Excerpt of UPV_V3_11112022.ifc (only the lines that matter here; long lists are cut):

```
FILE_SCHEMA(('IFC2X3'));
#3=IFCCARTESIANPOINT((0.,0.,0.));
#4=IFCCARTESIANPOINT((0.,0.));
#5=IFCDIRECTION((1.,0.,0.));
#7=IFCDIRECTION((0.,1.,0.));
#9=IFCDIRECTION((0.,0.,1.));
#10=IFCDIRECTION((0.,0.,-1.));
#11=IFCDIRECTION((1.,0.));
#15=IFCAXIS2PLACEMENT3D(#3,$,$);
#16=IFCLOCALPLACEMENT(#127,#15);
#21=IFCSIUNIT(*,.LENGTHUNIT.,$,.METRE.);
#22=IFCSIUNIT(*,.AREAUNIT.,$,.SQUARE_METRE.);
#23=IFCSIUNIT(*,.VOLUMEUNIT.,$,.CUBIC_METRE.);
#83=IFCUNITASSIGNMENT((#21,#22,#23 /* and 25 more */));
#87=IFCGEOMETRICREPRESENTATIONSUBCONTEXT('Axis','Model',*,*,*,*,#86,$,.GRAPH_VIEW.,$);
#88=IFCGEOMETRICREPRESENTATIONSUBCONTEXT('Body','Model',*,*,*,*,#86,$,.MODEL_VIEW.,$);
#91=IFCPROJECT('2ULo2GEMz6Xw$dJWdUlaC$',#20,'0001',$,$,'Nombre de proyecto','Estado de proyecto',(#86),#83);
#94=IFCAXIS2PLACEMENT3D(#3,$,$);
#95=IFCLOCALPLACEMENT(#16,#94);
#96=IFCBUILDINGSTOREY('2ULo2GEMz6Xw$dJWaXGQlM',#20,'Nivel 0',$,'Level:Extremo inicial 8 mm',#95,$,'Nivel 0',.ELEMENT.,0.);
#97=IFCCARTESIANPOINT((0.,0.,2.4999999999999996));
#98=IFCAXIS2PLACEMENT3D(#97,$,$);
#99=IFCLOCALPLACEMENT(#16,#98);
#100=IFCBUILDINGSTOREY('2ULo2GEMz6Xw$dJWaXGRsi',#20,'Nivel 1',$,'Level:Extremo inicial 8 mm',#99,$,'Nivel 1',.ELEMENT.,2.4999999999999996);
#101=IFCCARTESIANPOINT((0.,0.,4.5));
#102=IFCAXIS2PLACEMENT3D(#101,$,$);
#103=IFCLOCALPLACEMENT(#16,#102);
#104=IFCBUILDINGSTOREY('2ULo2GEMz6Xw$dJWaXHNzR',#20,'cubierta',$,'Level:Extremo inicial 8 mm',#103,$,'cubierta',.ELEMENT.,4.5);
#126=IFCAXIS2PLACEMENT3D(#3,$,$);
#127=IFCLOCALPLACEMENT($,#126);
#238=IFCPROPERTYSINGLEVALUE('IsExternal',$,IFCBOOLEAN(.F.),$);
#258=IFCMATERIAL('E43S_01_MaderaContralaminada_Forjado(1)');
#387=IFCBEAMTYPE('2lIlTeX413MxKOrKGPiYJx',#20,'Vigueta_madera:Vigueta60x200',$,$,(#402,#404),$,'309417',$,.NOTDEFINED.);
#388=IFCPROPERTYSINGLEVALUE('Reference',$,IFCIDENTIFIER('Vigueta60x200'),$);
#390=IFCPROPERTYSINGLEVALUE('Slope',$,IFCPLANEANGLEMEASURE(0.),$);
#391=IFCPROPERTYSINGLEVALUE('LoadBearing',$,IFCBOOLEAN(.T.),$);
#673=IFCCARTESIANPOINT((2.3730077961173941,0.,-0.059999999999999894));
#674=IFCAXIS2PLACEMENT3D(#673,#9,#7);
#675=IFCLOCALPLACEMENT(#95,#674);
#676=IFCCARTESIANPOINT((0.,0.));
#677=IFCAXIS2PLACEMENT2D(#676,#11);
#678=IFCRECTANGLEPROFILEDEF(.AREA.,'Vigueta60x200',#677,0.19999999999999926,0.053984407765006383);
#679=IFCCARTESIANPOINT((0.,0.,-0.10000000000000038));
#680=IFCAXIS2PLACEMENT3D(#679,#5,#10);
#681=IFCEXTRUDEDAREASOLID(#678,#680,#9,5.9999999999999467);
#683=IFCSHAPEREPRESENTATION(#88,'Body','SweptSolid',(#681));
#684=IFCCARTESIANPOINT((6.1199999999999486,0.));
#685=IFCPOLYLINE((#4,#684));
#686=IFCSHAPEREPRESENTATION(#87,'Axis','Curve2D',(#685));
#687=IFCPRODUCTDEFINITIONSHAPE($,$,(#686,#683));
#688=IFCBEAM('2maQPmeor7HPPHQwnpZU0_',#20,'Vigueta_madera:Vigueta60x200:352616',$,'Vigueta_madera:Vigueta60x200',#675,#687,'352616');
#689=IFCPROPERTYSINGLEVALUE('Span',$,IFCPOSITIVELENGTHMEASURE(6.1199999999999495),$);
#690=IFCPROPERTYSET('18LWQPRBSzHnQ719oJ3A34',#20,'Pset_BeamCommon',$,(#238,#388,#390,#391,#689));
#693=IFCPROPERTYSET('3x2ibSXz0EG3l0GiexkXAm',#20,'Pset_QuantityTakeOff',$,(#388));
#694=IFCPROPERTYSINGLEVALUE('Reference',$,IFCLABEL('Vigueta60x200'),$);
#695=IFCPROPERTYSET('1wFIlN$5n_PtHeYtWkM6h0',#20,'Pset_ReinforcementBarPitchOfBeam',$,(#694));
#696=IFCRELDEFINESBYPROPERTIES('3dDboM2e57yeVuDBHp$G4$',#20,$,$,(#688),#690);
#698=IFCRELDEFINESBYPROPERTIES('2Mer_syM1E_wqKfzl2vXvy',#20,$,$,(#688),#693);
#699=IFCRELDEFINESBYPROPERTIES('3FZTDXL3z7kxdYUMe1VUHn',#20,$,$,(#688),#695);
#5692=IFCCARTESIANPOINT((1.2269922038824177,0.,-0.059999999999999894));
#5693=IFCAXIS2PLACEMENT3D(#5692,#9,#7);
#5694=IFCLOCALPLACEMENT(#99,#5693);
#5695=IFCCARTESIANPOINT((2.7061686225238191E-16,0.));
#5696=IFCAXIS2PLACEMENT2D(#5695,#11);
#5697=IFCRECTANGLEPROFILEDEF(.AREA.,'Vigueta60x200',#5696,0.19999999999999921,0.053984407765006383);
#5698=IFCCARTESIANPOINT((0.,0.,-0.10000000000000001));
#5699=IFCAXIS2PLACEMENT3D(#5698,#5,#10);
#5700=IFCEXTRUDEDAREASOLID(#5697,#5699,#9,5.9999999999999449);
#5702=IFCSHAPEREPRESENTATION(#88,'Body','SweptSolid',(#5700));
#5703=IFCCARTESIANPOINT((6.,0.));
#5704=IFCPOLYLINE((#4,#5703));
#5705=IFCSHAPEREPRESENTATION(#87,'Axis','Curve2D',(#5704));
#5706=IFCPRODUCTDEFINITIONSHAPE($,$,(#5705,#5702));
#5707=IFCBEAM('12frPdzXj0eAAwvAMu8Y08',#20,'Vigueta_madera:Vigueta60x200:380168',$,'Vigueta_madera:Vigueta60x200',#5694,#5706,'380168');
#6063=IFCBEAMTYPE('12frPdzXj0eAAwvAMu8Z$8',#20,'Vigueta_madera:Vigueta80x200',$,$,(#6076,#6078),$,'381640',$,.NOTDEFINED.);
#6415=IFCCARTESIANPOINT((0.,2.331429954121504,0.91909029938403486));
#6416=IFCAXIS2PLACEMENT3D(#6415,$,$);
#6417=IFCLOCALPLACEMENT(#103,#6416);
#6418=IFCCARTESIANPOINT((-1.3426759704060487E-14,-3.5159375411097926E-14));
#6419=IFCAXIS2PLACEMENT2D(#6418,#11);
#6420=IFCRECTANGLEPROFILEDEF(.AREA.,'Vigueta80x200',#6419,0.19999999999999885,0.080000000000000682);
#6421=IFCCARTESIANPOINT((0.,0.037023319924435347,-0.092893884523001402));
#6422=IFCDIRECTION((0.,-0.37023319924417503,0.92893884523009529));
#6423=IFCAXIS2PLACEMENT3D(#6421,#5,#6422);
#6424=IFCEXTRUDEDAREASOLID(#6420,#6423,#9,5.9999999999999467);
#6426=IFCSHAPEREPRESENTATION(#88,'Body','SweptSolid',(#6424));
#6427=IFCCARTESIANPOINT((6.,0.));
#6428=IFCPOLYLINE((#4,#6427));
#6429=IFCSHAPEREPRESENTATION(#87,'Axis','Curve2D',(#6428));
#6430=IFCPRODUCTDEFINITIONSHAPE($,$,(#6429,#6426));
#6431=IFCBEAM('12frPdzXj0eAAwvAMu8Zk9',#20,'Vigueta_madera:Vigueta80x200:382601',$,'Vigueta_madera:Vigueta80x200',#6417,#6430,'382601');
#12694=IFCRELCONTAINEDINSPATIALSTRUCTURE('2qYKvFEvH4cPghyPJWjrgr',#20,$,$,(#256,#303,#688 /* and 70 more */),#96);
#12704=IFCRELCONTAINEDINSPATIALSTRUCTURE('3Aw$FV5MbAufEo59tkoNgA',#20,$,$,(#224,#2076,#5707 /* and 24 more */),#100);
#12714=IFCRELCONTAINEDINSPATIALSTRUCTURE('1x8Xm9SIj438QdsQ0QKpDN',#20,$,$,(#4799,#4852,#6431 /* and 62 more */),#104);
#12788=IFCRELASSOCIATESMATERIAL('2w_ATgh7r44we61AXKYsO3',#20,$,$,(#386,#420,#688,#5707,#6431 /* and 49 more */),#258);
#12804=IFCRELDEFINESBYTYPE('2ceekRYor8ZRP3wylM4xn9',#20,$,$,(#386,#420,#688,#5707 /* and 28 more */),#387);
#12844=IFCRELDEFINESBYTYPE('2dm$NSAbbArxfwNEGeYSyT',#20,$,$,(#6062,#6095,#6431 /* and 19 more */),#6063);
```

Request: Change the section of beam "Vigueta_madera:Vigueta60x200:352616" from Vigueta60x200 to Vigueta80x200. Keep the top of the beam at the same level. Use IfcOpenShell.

```python
import ifcopenshell
import ifcopenshell.api.pset
import ifcopenshell.api.type
import ifcopenshell.util.element
import ifcopenshell.util.representation

model = ifcopenshell.open("UPV_V3_11112022.ifc")

member = model.by_id(688)
source = next(p for p in model.by_type("IfcRectangleProfileDef") if p.ProfileName == "Vigueta80x200")

body = ifcopenshell.util.representation.get_representation(member, "Model", "Body")
solid = body.Items[0]
old_profile = solid.SweptArea

# Copy the section's sizes but keep this member's own profile position.
profile = ifcopenshell.util.element.copy(model, source)
# Profiles are centred, so shift by half the change in depth to hold the top.
shift = (old_profile.XDim - profile.XDim) / 2
x, y = old_profile.Position.Location.Coordinates
up = (-1.0, 0.0)  # upwards, in the solid's own plane
location = model.createIfcCartesianPoint((x + up[0] * shift, y + up[1] * shift))
profile.Position = model.createIfcAxis2Placement2D(location, old_profile.Position.RefDirection)
solid.SweptArea = profile
if not model.get_total_inverses(old_profile):
    ifcopenshell.util.element.remove_deep2(model, old_profile)

new_type = model.by_id(6063)
ifcopenshell.api.type.assign_type(
    model, related_objects=[member], relating_type=new_type, should_map_representations=False
)
member.Name = member.Name.replace("Vigueta60x200", "Vigueta80x200")
member.ObjectType = "Vigueta_madera:Vigueta80x200"
pset = model.by_id(ifcopenshell.util.element.get_pset(member, "Pset_BeamCommon", should_inherit=False)["id"])
ifcopenshell.api.pset.edit_pset(model, pset=pset, properties={"Reference": "Vigueta80x200"})
pset = model.by_id(ifcopenshell.util.element.get_pset(member, "Pset_QuantityTakeOff", should_inherit=False)["id"])
ifcopenshell.api.pset.edit_pset(model, pset=pset, properties={"Reference": "Vigueta80x200"})
pset = model.by_id(ifcopenshell.util.element.get_pset(member, "Pset_ReinforcementBarPitchOfBeam", should_inherit=False)["id"])
ifcopenshell.api.pset.edit_pset(model, pset=pset, properties={"Reference": "Vigueta80x200"})

print(solid.SweptArea)

model.write("UPV_V3_11112022_rev.ifc")
```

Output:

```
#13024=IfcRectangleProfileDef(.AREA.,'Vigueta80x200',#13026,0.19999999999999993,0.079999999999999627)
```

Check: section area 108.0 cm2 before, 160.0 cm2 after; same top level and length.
